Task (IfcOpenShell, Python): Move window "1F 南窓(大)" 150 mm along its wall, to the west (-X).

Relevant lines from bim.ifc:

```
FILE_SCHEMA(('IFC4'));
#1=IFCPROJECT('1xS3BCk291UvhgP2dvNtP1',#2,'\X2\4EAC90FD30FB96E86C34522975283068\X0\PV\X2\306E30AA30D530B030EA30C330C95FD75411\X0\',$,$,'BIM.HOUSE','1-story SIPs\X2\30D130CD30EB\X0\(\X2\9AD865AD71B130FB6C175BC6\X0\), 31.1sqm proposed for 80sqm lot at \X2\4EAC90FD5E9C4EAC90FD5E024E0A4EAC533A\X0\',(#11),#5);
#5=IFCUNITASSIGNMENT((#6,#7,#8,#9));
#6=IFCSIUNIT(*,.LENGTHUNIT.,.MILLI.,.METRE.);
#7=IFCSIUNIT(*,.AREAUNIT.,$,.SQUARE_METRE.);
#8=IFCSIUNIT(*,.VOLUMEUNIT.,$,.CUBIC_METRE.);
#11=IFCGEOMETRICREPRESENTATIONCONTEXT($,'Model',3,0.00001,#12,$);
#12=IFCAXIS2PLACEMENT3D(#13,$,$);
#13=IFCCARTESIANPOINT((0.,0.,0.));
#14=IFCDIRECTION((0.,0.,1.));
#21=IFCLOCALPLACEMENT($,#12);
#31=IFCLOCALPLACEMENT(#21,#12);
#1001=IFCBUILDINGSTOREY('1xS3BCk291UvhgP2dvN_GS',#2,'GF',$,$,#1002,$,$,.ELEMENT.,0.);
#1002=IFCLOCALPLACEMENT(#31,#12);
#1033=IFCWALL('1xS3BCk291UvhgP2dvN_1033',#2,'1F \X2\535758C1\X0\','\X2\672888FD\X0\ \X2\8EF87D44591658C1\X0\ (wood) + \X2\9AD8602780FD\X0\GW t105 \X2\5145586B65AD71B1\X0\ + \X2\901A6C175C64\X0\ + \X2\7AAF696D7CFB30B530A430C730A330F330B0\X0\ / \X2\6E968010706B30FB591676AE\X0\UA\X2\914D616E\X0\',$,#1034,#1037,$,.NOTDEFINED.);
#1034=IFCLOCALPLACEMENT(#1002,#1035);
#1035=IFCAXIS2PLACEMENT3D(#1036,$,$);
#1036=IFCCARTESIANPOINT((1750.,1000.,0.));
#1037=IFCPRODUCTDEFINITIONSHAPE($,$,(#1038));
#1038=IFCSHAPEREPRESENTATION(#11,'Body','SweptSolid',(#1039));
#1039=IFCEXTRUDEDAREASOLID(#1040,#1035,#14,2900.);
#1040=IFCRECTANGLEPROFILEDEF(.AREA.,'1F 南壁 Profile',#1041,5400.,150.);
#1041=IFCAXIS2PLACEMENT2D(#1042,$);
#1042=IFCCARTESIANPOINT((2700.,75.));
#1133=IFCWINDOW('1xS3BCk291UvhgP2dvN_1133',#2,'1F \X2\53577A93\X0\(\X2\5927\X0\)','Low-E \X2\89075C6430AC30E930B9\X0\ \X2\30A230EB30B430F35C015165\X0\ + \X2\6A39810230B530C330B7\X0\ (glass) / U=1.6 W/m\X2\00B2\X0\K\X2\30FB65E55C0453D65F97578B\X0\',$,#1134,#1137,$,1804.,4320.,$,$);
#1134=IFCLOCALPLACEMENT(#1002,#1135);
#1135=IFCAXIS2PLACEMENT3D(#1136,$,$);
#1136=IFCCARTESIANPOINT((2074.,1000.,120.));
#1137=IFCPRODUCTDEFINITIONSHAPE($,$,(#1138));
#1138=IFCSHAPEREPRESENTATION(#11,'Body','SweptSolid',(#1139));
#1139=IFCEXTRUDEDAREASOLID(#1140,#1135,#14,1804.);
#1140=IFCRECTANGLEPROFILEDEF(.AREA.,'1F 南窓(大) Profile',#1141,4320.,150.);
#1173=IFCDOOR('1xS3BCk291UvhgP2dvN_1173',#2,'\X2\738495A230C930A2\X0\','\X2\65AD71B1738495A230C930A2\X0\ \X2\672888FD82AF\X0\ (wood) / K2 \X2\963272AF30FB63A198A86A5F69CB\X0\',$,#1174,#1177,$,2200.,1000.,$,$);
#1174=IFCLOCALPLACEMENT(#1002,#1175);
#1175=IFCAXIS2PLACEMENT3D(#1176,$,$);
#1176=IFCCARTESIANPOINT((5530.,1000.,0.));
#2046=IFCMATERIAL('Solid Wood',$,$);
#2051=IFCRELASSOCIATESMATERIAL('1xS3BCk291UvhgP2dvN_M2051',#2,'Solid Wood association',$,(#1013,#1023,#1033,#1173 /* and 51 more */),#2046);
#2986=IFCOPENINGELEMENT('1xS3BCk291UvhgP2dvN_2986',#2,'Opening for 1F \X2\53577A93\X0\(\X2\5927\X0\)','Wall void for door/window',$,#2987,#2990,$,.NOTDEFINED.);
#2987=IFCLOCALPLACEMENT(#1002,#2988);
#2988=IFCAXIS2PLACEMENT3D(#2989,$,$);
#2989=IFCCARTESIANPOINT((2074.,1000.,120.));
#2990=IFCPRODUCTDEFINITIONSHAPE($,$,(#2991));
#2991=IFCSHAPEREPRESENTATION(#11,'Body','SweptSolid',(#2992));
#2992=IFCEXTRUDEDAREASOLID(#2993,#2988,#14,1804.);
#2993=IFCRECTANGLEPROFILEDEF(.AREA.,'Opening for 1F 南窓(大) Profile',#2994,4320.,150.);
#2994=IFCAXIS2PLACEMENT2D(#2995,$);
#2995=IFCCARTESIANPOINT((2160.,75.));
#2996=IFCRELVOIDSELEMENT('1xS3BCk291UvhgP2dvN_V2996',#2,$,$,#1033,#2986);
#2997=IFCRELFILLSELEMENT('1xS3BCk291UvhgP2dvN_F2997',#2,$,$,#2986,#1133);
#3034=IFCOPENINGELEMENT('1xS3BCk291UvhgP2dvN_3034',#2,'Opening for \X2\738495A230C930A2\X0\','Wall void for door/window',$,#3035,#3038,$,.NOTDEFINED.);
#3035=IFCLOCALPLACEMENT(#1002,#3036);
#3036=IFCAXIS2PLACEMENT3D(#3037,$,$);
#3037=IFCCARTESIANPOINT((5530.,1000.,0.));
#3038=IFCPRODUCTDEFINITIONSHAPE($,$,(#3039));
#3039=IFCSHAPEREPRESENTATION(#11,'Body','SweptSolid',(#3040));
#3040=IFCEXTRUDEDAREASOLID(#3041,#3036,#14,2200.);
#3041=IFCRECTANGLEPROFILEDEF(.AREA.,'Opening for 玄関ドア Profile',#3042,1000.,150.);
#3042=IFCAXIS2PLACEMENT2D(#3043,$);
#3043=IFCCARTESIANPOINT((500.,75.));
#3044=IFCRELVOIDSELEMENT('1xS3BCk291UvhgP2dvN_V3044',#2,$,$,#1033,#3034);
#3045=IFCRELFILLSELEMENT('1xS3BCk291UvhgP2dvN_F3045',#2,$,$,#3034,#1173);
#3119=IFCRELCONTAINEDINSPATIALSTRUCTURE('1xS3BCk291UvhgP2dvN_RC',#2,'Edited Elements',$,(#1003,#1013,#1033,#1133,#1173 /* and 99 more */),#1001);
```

```python
import ifcopenshell
import ifcopenshell.api.geometry
import ifcopenshell.util.placement
import ifcopenshell.util.unit

model = ifcopenshell.open("bim.ifc")
unit_scale = ifcopenshell.util.unit.calculate_unit_scale(model)

window = model.by_guid("1xS3BCk291UvhgP2dvN_1133")
opening = window.FillsVoids[0].RelatingOpeningElement
wall = opening.VoidsElements[0].RelatingBuildingElement

wall_matrix = ifcopenshell.util.placement.get_local_placement(wall.ObjectPlacement)
shift = wall_matrix[:3, 0] * -0.15 / unit_scale
before = ifcopenshell.util.placement.get_local_placement(window.ObjectPlacement)[:3, 3].copy()

# The window is not placed relative to its opening, so move both.
for product in (opening, window):
    matrix = ifcopenshell.util.placement.get_local_placement(product.ObjectPlacement)
    matrix[:3, 3] += shift
    ifcopenshell.api.geometry.edit_object_placement(model, product=product, matrix=matrix, is_si=False)

after = ifcopenshell.util.placement.get_local_placement(window.ObjectPlacement)[:3, 3]
print("window moved by", (after - before).round(3) + 0.0)

model.write("bim_updated.ifc")
```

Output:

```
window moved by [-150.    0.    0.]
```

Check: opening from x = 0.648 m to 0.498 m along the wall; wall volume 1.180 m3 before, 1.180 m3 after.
